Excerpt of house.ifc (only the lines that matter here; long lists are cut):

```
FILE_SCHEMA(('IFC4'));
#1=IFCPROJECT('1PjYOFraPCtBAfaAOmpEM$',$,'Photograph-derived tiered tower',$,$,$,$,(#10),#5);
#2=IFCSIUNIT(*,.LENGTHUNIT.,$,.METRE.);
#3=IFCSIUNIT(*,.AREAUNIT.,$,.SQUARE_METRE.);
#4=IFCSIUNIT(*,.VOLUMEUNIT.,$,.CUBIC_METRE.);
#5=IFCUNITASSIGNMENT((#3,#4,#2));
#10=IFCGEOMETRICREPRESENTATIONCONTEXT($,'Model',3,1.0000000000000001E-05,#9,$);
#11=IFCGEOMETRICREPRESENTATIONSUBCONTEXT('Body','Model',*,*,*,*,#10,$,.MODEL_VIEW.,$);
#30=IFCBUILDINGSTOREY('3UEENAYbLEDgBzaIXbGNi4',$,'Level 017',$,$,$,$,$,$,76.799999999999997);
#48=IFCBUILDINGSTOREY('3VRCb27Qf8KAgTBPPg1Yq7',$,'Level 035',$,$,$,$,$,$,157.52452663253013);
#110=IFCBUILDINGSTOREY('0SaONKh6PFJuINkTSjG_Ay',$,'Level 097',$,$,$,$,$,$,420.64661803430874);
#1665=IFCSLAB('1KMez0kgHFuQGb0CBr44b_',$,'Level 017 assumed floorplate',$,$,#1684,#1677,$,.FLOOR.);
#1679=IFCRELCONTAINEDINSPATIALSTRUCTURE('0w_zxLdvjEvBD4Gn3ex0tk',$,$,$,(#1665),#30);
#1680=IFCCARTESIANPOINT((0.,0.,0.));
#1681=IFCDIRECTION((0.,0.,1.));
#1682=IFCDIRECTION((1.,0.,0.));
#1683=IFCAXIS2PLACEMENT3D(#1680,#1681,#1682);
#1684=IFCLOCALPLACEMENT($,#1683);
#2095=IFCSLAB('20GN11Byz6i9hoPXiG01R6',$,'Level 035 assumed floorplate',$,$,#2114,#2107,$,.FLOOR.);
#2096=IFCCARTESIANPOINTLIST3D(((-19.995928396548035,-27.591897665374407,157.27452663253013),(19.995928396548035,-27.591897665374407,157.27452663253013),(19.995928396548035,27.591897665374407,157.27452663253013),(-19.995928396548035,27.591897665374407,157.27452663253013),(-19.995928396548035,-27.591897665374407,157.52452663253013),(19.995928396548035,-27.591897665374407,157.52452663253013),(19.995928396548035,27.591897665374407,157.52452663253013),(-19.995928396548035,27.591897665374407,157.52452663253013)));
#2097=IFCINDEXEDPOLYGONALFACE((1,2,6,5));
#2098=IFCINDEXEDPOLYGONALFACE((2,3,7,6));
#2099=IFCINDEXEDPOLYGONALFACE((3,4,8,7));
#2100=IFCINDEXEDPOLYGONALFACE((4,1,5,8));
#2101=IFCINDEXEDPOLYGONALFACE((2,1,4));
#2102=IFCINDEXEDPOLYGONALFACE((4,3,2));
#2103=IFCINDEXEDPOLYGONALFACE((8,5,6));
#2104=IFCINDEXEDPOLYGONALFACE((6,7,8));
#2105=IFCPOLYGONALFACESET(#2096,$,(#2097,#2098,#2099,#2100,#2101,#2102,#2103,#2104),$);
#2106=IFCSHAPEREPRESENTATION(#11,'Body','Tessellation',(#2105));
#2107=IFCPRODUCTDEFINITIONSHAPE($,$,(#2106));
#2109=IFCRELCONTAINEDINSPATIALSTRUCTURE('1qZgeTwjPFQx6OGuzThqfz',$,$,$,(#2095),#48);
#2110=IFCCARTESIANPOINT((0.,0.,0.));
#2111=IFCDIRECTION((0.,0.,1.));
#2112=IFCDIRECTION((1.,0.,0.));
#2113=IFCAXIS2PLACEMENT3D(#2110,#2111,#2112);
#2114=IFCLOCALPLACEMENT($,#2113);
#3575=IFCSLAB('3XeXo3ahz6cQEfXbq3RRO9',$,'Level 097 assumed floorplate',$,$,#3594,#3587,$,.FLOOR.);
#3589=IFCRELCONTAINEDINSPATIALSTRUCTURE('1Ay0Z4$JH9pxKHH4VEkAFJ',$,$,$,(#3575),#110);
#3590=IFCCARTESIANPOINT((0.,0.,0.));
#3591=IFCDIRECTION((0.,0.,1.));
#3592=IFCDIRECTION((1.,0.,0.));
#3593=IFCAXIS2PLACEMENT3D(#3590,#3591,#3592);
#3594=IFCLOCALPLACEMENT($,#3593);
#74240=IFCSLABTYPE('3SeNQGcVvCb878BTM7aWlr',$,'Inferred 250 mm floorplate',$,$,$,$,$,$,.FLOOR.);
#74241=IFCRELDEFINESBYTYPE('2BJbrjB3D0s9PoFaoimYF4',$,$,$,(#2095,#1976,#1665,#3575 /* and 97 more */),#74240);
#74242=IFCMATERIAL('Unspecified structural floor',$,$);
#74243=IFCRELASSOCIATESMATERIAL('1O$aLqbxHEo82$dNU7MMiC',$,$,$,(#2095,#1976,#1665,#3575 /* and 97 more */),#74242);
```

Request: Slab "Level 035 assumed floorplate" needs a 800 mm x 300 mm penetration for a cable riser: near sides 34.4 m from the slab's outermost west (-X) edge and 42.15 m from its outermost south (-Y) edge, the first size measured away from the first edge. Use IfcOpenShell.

```python
import numpy as np
import ifcopenshell
import ifcopenshell.api.feature
import ifcopenshell.api.geometry
import ifcopenshell.api.root
import ifcopenshell.geom
import ifcopenshell.util.placement
import ifcopenshell.util.representation
import ifcopenshell.util.shape
import ifcopenshell.util.unit

model = ifcopenshell.open("house.ifc")
unit_scale = ifcopenshell.util.unit.calculate_unit_scale(model)
settings = ifcopenshell.geom.settings()


def volume(element):
    """Net volume in cubic metres, openings subtracted."""
    shape = ifcopenshell.geom.create_shape(settings, element)
    return ifcopenshell.util.shape.get_volume(shape.geometry)


slab = model.by_guid("20GN11Byz6i9hoPXiG01R6")
before = volume(slab)

# Extent in the slab's own axes, in metres. The edges named are its -X and -Y sides.
slab_shape = ifcopenshell.geom.create_shape(settings, slab)
vertices = ifcopenshell.util.shape.get_vertices(slab_shape.geometry)
x_min, y_min, bottom = vertices.min(axis=0)
top = vertices[:, 2].max()

opening = ifcopenshell.api.root.create_entity(model, ifc_class="IfcOpeningElement", name="Cable riser opening", predefined_type="OPENING")
context = ifcopenshell.util.representation.get_context(model, "Model", "Body", "MODEL_VIEW")
width, depth = 0.8, 0.3
outline = [(0.0, 0.0), (width, 0.0), (width, depth), (0.0, depth), (0.0, 0.0)]
# Overshoot both faces by 50 mm so the cut is clean.
shape = ifcopenshell.api.geometry.add_slab_representation(
    model, context=context, depth=top - bottom + 0.1, polyline=outline
)
ifcopenshell.api.geometry.assign_representation(model, product=opening, representation=shape)

matrix = ifcopenshell.util.placement.get_local_placement(slab.ObjectPlacement)
matrix[:, 3] = matrix @ np.append(np.array([x_min + 34.4, y_min + 42.15, bottom - 0.05]) / unit_scale, 1.0)
ifcopenshell.api.geometry.edit_object_placement(model, product=opening, matrix=matrix, is_si=False)
ifcopenshell.api.feature.add_feature(model, feature=opening, element=slab)

after = volume(slab)

print(f"slab volume {before:.3f} -> {after:.3f} m3")

model.write("house-out.ifc")
```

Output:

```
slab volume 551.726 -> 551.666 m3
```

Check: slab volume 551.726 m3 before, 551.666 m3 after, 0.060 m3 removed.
